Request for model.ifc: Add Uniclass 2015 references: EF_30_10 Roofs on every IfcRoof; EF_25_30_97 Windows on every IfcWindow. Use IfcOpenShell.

First a look at what the model holds.

```python
import ifcopenshell

model = ifcopenshell.open("model.ifc")
print(model.schema)
print("classifications:", [c.Name for c in model.by_type("IfcClassification")])
for ifc_class in ("IfcDoor", "IfcRoof", "IfcStair", "IfcWall", "IfcWindow"):
    print(ifc_class, len(model.by_type(ifc_class)))
```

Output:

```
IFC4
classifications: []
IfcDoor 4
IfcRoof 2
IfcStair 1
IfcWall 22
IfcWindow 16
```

```python
import ifcopenshell
import ifcopenshell.api.classification

model = ifcopenshell.open("model.ifc")

system = ifcopenshell.api.classification.add_classification(model, classification="Uniclass 2015")

codes = {
    "IfcRoof": ("EF_30_10", "Roofs"),
    "IfcWindow": ("EF_25_30_97", "Windows"),
}
for ifc_class, (code, name) in codes.items():
    products = model.by_type(ifc_class)
    ifcopenshell.api.classification.add_reference(
        model, products=products, classification=system, identification=code, name=name
    )
    print(code, len(products))

model.write("model-out.ifc")
```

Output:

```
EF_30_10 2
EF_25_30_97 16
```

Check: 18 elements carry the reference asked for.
